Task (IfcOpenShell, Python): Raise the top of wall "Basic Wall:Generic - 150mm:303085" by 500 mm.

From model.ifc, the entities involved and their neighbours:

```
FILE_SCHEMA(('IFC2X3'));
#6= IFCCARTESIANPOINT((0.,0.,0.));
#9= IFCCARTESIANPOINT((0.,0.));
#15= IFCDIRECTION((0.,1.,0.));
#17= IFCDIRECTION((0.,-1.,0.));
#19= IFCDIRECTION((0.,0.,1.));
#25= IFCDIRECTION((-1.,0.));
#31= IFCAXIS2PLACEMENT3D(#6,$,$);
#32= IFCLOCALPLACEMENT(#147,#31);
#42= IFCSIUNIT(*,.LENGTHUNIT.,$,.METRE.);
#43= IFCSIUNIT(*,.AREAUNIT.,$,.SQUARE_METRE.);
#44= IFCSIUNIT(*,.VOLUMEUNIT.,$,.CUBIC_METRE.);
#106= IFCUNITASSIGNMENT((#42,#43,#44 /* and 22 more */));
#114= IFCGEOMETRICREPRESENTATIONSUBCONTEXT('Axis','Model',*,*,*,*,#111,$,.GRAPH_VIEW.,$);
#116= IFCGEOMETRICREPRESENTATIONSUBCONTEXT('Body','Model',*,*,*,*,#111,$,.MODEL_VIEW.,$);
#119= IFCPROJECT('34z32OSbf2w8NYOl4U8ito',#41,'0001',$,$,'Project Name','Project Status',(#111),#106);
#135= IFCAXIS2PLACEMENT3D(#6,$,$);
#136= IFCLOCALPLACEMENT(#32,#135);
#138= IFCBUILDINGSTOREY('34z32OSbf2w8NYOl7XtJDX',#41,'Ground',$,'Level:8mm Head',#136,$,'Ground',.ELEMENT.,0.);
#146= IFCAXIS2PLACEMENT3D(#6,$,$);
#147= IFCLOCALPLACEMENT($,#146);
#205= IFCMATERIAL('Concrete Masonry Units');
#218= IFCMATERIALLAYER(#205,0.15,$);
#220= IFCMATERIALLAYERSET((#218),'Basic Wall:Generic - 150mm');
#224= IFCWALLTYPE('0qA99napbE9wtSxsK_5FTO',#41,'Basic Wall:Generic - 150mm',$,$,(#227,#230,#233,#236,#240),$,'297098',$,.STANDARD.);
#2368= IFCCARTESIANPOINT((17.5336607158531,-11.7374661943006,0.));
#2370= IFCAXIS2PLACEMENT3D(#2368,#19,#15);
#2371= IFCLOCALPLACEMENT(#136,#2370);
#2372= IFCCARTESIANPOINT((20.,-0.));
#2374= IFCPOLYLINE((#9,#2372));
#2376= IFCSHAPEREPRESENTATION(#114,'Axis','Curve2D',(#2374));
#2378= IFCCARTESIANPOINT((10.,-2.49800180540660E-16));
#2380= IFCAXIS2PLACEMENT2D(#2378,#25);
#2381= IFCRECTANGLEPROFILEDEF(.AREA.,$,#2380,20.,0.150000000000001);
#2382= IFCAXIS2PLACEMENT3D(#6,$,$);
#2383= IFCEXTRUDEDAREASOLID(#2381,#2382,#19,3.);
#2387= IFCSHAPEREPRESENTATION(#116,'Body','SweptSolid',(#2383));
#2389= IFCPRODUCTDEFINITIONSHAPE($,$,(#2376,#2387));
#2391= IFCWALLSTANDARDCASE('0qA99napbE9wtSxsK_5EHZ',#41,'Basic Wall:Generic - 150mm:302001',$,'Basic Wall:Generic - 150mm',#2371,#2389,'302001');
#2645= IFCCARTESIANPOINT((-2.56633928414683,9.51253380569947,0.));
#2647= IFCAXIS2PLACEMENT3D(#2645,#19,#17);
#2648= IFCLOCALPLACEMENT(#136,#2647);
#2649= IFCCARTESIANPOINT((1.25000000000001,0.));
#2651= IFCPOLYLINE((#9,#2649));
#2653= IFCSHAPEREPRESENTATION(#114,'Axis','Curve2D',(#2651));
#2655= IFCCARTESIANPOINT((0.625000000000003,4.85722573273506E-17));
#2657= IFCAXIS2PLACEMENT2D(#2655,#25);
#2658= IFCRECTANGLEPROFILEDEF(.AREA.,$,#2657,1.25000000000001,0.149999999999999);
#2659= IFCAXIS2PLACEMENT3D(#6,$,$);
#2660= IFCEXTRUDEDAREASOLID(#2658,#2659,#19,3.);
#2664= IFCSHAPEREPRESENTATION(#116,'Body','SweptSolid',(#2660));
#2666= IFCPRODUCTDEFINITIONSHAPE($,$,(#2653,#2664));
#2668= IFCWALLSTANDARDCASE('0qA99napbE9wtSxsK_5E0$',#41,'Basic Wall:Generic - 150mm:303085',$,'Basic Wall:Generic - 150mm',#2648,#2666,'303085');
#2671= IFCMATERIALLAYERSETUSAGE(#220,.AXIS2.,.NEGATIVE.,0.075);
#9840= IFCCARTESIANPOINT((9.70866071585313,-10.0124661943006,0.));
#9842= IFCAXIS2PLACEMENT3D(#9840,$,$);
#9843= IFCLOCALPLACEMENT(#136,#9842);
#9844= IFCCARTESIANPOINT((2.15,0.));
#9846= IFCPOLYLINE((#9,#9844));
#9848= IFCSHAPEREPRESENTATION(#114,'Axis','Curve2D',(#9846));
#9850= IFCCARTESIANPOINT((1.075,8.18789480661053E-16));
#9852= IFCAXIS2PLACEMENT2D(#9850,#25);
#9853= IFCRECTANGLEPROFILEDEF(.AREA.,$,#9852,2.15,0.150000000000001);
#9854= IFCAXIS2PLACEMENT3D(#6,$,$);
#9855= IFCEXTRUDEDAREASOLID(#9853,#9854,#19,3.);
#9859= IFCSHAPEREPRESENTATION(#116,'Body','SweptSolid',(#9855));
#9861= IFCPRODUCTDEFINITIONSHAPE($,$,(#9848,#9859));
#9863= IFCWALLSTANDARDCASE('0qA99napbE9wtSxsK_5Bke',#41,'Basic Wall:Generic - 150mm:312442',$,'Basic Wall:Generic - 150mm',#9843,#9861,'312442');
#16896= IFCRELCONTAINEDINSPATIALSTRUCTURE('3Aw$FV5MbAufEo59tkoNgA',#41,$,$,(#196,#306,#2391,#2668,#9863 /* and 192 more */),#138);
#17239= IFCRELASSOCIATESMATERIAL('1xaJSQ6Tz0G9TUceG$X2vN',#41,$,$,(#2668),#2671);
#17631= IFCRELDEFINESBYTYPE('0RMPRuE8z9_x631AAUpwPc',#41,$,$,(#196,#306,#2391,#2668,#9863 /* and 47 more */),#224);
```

```python
import ifcopenshell
import ifcopenshell.geom
import ifcopenshell.util.representation
import ifcopenshell.util.shape
import ifcopenshell.util.unit

model = ifcopenshell.open("model.ifc")
unit_scale = ifcopenshell.util.unit.calculate_unit_scale(model)
settings = ifcopenshell.geom.settings()


def volume(element):
    """Net volume in cubic metres, openings subtracted."""
    shape = ifcopenshell.geom.create_shape(settings, element)
    return ifcopenshell.util.shape.get_volume(shape.geometry)


wall = model.by_guid("0qA99napbE9wtSxsK_5E0$")
before = volume(wall)

body = ifcopenshell.util.representation.get_representation(wall, "Model", "Body")
solid = body.Items[0]
old_height = solid.Depth
solid.Depth += 0.5 / unit_scale
after = volume(wall)

print(f"height {old_height:g} -> {solid.Depth:g}, volume {before:.3f} -> {after:.3f} m3")

model.write("model_updated.ifc")
```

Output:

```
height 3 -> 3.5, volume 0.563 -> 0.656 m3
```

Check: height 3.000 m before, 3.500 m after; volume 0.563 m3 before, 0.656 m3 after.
